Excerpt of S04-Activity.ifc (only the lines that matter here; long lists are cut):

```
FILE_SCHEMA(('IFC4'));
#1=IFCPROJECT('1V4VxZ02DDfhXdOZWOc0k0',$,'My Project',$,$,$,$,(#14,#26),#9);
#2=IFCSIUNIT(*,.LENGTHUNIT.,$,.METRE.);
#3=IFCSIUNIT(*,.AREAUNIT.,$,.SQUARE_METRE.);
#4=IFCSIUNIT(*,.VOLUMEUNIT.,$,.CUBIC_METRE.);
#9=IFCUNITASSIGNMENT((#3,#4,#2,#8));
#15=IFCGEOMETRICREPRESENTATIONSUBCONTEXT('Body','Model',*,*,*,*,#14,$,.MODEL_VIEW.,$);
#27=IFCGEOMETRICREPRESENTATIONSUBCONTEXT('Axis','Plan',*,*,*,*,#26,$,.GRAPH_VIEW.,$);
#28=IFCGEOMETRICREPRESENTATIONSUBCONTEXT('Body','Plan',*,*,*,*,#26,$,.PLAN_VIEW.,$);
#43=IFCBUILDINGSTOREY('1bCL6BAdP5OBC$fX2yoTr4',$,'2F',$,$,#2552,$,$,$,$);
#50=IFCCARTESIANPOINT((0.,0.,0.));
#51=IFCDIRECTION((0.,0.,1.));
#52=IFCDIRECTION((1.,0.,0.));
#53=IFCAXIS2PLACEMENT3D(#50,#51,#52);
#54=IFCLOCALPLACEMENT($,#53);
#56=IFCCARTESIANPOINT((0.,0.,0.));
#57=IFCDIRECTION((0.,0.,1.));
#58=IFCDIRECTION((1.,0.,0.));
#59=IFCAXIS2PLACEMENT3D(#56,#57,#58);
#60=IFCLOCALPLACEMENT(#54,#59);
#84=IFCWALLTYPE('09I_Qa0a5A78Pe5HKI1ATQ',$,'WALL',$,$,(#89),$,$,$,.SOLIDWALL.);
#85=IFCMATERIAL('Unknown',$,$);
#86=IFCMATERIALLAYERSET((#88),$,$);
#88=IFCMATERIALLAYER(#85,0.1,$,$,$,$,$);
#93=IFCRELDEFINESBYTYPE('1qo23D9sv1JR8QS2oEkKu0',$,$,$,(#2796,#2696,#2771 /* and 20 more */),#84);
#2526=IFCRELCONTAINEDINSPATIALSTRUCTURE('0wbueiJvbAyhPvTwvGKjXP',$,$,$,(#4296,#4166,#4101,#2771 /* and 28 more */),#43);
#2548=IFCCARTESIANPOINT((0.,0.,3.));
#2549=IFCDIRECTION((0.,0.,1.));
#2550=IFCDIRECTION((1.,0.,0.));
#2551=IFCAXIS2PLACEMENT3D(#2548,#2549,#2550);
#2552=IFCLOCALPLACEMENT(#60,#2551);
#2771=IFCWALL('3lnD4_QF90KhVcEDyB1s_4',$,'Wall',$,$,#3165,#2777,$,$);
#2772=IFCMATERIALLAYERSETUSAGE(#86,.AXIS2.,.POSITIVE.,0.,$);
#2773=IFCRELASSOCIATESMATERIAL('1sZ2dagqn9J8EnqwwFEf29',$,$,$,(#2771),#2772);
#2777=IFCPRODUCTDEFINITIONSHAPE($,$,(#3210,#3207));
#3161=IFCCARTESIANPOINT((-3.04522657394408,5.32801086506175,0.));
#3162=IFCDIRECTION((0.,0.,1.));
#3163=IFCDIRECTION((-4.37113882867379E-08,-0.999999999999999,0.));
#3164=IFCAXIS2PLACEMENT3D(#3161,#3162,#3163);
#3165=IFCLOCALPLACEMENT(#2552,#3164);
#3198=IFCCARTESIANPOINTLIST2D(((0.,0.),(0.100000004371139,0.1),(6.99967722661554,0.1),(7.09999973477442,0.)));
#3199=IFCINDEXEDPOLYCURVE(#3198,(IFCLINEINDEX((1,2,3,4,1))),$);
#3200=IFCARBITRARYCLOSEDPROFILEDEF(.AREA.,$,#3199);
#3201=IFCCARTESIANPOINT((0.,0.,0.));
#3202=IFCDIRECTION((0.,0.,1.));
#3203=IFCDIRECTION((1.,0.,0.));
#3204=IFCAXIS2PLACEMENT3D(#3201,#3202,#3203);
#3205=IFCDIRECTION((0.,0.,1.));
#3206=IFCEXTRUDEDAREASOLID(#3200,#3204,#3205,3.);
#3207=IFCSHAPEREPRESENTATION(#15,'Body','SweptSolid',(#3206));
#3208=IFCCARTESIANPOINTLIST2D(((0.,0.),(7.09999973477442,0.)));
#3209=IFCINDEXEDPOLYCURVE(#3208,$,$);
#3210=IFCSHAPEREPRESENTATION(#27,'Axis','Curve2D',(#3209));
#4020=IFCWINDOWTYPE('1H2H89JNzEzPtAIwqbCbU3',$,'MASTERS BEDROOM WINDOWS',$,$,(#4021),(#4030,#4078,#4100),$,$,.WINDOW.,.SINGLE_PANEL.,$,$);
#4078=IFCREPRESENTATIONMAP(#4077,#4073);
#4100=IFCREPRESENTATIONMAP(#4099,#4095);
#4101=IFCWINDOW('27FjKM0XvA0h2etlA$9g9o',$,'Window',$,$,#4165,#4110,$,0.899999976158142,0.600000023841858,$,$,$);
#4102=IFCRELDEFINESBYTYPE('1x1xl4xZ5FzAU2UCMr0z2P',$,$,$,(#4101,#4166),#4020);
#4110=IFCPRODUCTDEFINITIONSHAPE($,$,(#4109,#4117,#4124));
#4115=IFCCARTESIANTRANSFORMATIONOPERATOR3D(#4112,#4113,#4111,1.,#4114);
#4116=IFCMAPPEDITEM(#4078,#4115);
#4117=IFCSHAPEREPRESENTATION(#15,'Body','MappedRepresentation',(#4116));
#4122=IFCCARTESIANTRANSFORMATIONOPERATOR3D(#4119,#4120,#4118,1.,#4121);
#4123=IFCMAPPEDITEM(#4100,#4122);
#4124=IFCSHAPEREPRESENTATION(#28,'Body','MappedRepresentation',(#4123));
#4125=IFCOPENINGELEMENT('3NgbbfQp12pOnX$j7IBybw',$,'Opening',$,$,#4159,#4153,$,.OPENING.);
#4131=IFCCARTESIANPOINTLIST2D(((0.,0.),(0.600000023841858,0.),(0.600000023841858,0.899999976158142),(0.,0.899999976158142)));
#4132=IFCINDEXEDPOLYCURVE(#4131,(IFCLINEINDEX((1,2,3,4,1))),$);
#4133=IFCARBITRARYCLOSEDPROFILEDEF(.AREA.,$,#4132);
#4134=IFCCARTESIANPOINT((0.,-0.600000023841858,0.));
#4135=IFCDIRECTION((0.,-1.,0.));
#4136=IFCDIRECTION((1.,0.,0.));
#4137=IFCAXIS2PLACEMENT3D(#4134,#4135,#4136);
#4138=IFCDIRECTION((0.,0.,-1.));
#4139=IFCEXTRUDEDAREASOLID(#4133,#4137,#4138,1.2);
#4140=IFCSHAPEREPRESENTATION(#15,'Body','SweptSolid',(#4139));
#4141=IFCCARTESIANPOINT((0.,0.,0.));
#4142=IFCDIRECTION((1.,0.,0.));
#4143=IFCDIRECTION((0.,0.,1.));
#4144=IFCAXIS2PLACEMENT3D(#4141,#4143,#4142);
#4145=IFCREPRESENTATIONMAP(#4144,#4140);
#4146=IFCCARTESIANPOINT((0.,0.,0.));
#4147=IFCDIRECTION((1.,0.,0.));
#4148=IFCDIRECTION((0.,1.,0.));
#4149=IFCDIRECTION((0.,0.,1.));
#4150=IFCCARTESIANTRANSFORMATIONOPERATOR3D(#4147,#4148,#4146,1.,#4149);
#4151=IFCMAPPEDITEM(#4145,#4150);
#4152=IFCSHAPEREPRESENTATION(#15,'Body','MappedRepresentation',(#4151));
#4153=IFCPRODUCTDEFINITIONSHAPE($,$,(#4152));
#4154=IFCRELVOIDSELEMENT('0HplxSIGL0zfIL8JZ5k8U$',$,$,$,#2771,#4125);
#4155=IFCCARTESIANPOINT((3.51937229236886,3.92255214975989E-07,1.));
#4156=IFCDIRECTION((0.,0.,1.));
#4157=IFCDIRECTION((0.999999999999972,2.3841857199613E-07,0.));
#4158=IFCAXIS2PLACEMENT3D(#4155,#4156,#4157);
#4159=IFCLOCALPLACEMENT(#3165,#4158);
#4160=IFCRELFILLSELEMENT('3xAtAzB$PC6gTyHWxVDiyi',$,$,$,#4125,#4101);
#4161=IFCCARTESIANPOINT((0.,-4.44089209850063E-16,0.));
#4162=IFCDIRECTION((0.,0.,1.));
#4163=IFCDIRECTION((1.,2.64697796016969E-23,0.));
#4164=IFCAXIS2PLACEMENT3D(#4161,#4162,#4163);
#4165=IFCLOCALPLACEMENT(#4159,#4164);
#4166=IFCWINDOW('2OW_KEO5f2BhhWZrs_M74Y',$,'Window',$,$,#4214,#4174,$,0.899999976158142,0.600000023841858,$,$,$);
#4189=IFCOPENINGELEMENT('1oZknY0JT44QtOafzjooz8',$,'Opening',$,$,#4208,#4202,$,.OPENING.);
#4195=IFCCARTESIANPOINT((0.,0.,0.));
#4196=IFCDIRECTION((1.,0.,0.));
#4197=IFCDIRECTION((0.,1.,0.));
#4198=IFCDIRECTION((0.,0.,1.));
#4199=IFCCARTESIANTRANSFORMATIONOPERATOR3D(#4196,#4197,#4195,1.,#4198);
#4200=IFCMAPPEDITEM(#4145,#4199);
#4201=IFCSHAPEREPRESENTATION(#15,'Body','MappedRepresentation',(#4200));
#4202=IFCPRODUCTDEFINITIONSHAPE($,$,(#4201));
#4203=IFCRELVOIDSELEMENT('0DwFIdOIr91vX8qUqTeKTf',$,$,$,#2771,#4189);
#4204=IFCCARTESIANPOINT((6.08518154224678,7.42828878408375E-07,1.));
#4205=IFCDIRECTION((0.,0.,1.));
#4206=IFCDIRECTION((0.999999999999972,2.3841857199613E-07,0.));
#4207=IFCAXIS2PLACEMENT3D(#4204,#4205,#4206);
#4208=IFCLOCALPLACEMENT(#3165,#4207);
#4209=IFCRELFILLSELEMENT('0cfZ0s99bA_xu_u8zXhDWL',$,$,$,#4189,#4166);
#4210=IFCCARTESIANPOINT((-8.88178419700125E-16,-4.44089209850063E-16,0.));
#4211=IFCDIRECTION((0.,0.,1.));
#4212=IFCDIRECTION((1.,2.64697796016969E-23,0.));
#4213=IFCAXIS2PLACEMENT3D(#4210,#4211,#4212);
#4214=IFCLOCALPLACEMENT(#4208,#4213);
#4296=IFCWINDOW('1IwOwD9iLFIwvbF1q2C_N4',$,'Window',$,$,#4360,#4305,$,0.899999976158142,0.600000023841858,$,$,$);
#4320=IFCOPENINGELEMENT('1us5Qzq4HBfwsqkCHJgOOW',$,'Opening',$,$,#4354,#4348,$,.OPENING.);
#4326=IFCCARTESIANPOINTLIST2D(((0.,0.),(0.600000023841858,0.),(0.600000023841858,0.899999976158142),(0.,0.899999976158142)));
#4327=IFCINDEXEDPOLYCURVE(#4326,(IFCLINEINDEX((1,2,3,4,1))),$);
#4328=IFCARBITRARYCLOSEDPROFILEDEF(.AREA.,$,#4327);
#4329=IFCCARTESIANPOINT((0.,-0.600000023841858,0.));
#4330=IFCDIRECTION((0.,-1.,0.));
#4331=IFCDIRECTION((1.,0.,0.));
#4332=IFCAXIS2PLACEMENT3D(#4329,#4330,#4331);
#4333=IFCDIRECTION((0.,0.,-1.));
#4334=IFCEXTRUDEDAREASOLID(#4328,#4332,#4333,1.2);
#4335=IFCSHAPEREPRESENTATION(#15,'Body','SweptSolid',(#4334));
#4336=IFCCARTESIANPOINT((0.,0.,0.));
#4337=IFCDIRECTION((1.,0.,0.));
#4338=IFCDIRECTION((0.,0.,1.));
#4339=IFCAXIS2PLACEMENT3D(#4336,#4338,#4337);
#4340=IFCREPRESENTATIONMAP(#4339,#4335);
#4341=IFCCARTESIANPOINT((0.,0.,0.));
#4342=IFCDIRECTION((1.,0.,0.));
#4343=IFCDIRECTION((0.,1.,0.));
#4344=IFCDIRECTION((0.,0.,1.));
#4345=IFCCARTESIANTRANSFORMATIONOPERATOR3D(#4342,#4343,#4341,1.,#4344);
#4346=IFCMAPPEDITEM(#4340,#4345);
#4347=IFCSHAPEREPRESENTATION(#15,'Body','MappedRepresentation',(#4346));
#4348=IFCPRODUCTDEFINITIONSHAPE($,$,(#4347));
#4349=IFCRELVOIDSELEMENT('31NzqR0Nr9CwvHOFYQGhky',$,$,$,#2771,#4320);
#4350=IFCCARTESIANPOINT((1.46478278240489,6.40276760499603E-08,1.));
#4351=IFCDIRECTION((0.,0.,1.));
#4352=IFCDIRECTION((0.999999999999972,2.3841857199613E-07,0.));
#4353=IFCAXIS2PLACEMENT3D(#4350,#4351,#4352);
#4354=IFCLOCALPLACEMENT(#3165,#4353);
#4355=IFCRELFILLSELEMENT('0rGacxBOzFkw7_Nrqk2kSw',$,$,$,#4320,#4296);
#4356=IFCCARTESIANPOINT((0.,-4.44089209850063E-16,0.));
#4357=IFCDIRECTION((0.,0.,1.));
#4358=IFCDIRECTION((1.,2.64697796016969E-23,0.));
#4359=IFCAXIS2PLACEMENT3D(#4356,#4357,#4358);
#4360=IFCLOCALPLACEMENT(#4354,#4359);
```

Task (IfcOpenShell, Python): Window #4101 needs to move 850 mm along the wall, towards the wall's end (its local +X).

```python
import ifcopenshell
import ifcopenshell.api.geometry
import ifcopenshell.util.placement
import ifcopenshell.util.unit

model = ifcopenshell.open("S04-Activity.ifc")
unit_scale = ifcopenshell.util.unit.calculate_unit_scale(model)

window = model.by_guid("27FjKM0XvA0h2etlA$9g9o")
opening = window.FillsVoids[0].RelatingOpeningElement
wall = opening.VoidsElements[0].RelatingBuildingElement

wall_matrix = ifcopenshell.util.placement.get_local_placement(wall.ObjectPlacement)
shift = wall_matrix[:3, 0] * 0.85 / unit_scale
before = ifcopenshell.util.placement.get_local_placement(window.ObjectPlacement)[:3, 3].copy()

# The window is placed relative to its opening, so it follows when the opening moves.
matrix = ifcopenshell.util.placement.get_local_placement(opening.ObjectPlacement)
matrix[:3, 3] += shift
ifcopenshell.api.geometry.edit_object_placement(
    model, product=opening, matrix=matrix, is_si=False, should_transform_children=True
)

after = ifcopenshell.util.placement.get_local_placement(window.ObjectPlacement)[:3, 3]
print("window moved by", (after - before).round(3) + 0.0)

model.write("S04-Activity_rev.ifc")
```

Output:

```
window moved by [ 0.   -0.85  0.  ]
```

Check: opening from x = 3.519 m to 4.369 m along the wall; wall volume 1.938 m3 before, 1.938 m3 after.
